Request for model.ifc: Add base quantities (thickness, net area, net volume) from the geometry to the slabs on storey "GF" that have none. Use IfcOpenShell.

First a look at what the model holds.

```python
import ifcopenshell
import ifcopenshell.util.element
import ifcopenshell.util.unit

model = ifcopenshell.open("model.ifc")
print(model.schema)
for unit_type in ("LENGTHUNIT", "AREAUNIT", "VOLUMEUNIT"):
    print(unit_type, ifcopenshell.util.unit.calculate_unit_scale(model, unit_type))
storey = next(s for s in model.by_type("IfcBuildingStorey") if s.Name == "GF")
slabs = [e for e in ifcopenshell.util.element.get_decomposition(storey) if e.is_a("IfcSlab")]
for e in sorted(slabs, key=lambda e: e.id()):
    print(e.id(), e.is_a(), e.Name, list(ifcopenshell.util.element.get_psets(e, qtos_only=True)), sep=" | ")
```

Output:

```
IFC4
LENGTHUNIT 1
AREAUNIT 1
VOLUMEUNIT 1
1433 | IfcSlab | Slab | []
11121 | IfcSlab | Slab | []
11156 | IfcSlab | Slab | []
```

```python
import ifcopenshell
import ifcopenshell.api.pset
import ifcopenshell.geom
import ifcopenshell.util.element
import ifcopenshell.util.shape
import ifcopenshell.util.unit

model = ifcopenshell.open("model.ifc")
unit_scale = ifcopenshell.util.unit.calculate_unit_scale(model)
area_scale = ifcopenshell.util.unit.calculate_unit_scale(model, "AREAUNIT")
volume_scale = ifcopenshell.util.unit.calculate_unit_scale(model, "VOLUMEUNIT")
settings = ifcopenshell.geom.settings()

storey = next(s for s in model.by_type("IfcBuildingStorey") if s.Name == "GF")
slabs = [e for e in ifcopenshell.util.element.get_decomposition(storey) if e.is_a("IfcSlab")]

for e in sorted(slabs, key=lambda e: e.id()):
    if ifcopenshell.util.element.get_psets(e, qtos_only=True, should_inherit=False):
        continue
    # Geometry comes back in metres, in the element's own axes.
    shape = ifcopenshell.geom.create_shape(settings, e)
    values = {
        "Width": ifcopenshell.util.shape.get_z(shape.geometry) / unit_scale,
        "NetArea": ifcopenshell.util.shape.get_footprint_area(shape.geometry) / area_scale,
        "NetVolume": ifcopenshell.util.shape.get_volume(shape.geometry) / volume_scale,
    }
    qto = ifcopenshell.api.pset.add_qto(model, product=e, name="Qto_SlabBaseQuantities")
    ifcopenshell.api.pset.edit_qto(model, qto=qto, properties=values)
    print(e.id(), {k: round(v, 3) for k, v in values.items()})

model.write("model_edited.ifc")
```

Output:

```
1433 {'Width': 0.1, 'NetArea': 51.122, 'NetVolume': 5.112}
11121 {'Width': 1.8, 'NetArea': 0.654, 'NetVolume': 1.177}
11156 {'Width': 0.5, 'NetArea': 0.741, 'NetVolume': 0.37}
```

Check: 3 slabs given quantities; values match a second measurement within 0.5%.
